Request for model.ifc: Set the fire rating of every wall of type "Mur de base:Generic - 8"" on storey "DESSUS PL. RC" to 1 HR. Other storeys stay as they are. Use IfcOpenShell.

First a look at what the model holds.

```python
import ifcopenshell
import ifcopenshell.util.element

model = ifcopenshell.open("model.ifc")
print(model.schema)
storey = next(s for s in model.by_type("IfcBuildingStorey") if s.Name == "DESSUS PL. RC")
walls = [e for e in ifcopenshell.util.element.get_decomposition(storey) if e.is_a("IfcWall")]
seen = {}
for e in walls:
    element_type = ifcopenshell.util.element.get_type(e)
    key = (element_type.Name if element_type != e and element_type else None, ifcopenshell.util.element.get_pset(e, "Pset_WallCommon", "FireRating"))
    seen[key] = seen.get(key, 0) + 1
for (name, value), count in sorted(seen.items(), key=str):
    print(count, "x", name, "|", value)
```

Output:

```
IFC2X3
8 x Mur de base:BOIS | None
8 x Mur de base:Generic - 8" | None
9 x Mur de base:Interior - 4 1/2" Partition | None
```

```python
import ifcopenshell
import ifcopenshell.api.pset
import ifcopenshell.util.element

model = ifcopenshell.open("model.ifc")

storey = next(s for s in model.by_type("IfcBuildingStorey") if s.Name == "DESSUS PL. RC")
walls = [e for e in ifcopenshell.util.element.get_decomposition(storey) if e.is_a("IfcWall")]

count = 0
for e in walls:
    element_type = ifcopenshell.util.element.get_type(e)
    if element_type in (None, e) or element_type.Name != 'Mur de base:Generic - 8"':
        continue
    # add_pset returns the element's existing set when there is one.
    pset = ifcopenshell.api.pset.add_pset(model, product=e, name="Pset_WallCommon")
    ifcopenshell.api.pset.edit_pset(model, pset=pset, properties={"FireRating": "1 HR"})
    count += 1

print(count, "walls updated")

model.write("model_edited.ifc")
```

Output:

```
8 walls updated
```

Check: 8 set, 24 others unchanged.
